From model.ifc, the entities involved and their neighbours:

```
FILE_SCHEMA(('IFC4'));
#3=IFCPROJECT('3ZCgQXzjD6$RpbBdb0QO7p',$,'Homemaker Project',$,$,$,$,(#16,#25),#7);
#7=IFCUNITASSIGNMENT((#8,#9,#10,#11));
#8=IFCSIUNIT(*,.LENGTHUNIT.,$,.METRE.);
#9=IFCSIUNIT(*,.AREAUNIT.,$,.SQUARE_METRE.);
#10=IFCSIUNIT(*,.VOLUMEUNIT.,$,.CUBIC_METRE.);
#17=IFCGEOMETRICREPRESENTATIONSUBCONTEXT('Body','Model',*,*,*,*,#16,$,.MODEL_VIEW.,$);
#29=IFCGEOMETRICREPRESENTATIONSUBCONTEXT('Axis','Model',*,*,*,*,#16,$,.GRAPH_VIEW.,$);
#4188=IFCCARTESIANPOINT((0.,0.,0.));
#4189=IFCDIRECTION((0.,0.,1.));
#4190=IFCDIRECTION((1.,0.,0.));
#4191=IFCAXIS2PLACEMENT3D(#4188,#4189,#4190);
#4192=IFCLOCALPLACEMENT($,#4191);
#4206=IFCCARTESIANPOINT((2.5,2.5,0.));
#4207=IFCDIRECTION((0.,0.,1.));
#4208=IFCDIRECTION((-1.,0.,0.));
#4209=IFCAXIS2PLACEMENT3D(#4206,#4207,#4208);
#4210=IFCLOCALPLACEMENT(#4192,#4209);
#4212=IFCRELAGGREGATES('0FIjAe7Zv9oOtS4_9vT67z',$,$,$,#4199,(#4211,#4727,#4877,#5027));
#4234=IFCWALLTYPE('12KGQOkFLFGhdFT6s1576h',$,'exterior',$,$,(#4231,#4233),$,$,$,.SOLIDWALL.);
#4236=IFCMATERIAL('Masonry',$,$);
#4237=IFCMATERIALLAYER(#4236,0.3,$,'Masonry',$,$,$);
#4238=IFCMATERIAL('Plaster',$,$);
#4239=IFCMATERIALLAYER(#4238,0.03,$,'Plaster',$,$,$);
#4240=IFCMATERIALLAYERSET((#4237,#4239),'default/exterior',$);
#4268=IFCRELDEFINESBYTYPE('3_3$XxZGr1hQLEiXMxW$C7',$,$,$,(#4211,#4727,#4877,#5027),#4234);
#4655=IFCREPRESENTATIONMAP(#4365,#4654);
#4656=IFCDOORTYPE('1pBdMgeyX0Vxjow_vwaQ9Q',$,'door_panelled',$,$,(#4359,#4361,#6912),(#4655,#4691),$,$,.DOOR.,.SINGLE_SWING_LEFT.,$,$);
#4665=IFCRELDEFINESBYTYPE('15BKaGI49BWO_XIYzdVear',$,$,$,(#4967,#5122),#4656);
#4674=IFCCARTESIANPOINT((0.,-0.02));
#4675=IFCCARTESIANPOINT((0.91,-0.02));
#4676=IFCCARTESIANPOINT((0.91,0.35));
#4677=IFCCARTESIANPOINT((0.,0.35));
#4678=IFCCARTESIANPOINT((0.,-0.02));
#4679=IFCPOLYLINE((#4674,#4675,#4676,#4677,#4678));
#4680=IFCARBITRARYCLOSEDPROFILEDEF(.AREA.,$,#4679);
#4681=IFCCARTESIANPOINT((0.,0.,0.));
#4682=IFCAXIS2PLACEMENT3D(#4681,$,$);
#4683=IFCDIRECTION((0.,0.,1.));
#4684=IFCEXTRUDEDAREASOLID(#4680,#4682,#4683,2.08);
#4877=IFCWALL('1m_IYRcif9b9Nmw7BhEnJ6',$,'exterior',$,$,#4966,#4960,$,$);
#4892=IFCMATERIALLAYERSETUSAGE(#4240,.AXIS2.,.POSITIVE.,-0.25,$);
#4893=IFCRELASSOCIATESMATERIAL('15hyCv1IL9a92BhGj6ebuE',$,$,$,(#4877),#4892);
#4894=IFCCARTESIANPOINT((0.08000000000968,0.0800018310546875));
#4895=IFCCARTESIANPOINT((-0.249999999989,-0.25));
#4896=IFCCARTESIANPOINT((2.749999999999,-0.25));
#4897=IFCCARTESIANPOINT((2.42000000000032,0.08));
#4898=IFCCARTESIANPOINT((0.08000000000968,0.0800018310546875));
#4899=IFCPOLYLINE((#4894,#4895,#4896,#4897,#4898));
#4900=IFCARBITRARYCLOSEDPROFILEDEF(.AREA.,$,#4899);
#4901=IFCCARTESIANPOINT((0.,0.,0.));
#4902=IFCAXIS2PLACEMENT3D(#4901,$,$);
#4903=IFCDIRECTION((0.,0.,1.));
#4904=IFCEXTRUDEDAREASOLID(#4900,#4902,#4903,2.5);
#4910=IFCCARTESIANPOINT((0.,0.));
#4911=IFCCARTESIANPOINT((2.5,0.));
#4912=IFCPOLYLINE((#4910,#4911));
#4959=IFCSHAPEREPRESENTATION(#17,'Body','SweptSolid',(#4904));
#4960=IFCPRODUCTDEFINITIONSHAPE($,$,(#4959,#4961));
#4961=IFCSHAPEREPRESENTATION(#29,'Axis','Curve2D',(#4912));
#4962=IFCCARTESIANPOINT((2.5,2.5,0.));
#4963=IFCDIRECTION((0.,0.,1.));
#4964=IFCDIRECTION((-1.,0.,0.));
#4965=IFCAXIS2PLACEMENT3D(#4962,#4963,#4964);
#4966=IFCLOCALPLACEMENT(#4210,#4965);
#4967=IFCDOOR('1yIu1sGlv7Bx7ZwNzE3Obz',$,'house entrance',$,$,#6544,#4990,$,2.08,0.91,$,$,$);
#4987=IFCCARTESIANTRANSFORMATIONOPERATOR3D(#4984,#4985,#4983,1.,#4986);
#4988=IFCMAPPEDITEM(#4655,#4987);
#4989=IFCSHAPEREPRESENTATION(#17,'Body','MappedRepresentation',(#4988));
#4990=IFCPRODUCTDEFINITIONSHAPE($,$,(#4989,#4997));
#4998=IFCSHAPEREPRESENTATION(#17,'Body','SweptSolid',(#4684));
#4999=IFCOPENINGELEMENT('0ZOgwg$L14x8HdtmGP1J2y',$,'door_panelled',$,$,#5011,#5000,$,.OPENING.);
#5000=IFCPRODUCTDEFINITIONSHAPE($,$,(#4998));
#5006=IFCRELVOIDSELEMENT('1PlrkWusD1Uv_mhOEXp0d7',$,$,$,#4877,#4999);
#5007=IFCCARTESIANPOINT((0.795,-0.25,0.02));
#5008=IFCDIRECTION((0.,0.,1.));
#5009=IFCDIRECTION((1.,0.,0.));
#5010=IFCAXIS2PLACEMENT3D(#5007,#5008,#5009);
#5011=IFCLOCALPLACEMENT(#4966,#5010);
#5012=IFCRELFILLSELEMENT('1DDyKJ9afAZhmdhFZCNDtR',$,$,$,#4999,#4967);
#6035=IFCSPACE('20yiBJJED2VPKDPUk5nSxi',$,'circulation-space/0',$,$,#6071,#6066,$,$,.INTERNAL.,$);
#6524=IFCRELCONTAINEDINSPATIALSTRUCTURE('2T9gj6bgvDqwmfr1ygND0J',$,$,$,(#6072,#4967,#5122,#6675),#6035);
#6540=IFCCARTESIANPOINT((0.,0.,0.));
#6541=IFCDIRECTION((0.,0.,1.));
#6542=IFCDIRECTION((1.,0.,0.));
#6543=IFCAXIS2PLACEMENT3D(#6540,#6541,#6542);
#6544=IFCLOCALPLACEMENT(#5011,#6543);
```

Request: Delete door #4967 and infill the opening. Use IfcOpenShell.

```python
import ifcopenshell
import ifcopenshell.api.feature
import ifcopenshell.api.root
import ifcopenshell.geom
import ifcopenshell.util.shape

model = ifcopenshell.open("model.ifc")
settings = ifcopenshell.geom.settings()


def volume(element):
    """Net volume in cubic metres, openings subtracted."""
    shape = ifcopenshell.geom.create_shape(settings, element)
    return ifcopenshell.util.shape.get_volume(shape.geometry)


door = model.by_guid("1yIu1sGlv7Bx7ZwNzE3Obz")
opening = door.FillsVoids[0].RelatingOpeningElement
wall = opening.VoidsElements[0].RelatingBuildingElement
before = volume(wall)

ifcopenshell.api.root.remove_product(model, product=door)
ifcopenshell.api.feature.remove_feature(model, feature=opening)

after = volume(wall)

print(f"wall volume {before:.3f} -> {after:.3f} m3")

model.write("model-out.ifc")
```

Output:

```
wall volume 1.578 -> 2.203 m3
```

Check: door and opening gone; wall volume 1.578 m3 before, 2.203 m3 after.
